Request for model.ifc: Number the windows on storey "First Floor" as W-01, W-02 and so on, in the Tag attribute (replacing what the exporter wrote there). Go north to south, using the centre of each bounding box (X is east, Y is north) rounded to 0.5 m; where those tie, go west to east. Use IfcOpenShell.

First a look at what the model holds.

```python
import ifcopenshell
import ifcopenshell.util.element
import ifcopenshell.util.placement

model = ifcopenshell.open("model.ifc")
print(model.schema)
storey = next(s for s in model.by_type("IfcBuildingStorey") if s.Name == "First Floor")
windows = [e for e in ifcopenshell.util.element.get_decomposition(storey) if e.is_a("IfcWindow")]
for e in sorted(windows, key=lambda e: e.id()):
    origin = ifcopenshell.util.placement.get_local_placement(e.ObjectPlacement)[:3, 3]
    print(e.id(), e.Tag, e.Name, origin.round(2) + 0.0, sep=" | ")
```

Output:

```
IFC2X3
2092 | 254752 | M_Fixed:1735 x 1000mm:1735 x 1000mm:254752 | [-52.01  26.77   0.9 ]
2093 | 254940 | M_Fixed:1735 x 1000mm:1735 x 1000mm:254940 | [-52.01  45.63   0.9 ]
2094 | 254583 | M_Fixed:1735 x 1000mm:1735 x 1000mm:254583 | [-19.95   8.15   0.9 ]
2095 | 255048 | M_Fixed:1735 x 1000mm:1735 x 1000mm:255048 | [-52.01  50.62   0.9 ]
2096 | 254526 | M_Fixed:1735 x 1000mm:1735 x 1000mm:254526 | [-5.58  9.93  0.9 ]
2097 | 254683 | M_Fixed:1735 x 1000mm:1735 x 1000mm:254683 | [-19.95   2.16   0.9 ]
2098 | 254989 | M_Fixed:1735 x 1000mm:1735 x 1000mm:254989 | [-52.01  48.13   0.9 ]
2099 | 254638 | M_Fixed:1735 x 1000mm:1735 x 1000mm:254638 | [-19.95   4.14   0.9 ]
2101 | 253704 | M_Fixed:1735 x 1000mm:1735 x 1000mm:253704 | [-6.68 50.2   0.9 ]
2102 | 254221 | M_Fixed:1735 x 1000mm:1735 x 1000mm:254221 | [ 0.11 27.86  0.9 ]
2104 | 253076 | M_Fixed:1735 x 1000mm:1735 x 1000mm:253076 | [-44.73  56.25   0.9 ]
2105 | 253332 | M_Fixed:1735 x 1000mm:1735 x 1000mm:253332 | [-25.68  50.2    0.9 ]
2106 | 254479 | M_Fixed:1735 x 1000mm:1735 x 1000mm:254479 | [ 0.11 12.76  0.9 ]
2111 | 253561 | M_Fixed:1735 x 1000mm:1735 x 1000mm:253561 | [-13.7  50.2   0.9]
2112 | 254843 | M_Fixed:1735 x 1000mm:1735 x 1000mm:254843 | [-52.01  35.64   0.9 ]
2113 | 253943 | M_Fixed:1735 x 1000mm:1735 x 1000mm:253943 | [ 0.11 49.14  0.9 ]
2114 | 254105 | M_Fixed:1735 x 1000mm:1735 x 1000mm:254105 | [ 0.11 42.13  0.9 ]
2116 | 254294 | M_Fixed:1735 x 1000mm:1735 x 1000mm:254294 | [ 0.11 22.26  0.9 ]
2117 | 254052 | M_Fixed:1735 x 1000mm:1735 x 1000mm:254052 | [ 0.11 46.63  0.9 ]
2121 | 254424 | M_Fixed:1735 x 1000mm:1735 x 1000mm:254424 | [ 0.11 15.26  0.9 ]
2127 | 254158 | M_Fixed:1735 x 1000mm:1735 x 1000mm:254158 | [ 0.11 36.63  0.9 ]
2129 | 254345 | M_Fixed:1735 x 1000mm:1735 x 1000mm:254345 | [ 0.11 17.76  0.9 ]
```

```python
import ifcopenshell
import ifcopenshell.geom
import ifcopenshell.util.element
import ifcopenshell.util.shape

model = ifcopenshell.open("model.ifc")
settings = ifcopenshell.geom.settings()
settings.set("use-world-coords", True)


def centre(element):
    shape = ifcopenshell.geom.create_shape(settings, element)
    return ifcopenshell.util.shape.get_bbox_centroid(shape.geometry)


storey = next(s for s in model.by_type("IfcBuildingStorey") if s.Name == "First Floor")
windows = [e for e in ifcopenshell.util.element.get_decomposition(storey) if e.is_a("IfcWindow")]

# Insertion points can sit at a corner or the storey origin, so sort by the geometry (in metres).
centres = {e: centre(e) for e in windows}
windows.sort(key=lambda e: (-round(centres[e][1] / 0.5), centres[e][0]))

for i, e in enumerate(windows, start=1):
    number = f"W-{i:02d}"
    e.Tag = number
    print(e.id(), number)

model.write("model-out.ifc")
```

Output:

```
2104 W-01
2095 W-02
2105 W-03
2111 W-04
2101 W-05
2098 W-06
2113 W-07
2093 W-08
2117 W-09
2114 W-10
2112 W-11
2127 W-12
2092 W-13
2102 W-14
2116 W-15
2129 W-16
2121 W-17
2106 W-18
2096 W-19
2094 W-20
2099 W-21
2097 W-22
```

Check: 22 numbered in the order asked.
